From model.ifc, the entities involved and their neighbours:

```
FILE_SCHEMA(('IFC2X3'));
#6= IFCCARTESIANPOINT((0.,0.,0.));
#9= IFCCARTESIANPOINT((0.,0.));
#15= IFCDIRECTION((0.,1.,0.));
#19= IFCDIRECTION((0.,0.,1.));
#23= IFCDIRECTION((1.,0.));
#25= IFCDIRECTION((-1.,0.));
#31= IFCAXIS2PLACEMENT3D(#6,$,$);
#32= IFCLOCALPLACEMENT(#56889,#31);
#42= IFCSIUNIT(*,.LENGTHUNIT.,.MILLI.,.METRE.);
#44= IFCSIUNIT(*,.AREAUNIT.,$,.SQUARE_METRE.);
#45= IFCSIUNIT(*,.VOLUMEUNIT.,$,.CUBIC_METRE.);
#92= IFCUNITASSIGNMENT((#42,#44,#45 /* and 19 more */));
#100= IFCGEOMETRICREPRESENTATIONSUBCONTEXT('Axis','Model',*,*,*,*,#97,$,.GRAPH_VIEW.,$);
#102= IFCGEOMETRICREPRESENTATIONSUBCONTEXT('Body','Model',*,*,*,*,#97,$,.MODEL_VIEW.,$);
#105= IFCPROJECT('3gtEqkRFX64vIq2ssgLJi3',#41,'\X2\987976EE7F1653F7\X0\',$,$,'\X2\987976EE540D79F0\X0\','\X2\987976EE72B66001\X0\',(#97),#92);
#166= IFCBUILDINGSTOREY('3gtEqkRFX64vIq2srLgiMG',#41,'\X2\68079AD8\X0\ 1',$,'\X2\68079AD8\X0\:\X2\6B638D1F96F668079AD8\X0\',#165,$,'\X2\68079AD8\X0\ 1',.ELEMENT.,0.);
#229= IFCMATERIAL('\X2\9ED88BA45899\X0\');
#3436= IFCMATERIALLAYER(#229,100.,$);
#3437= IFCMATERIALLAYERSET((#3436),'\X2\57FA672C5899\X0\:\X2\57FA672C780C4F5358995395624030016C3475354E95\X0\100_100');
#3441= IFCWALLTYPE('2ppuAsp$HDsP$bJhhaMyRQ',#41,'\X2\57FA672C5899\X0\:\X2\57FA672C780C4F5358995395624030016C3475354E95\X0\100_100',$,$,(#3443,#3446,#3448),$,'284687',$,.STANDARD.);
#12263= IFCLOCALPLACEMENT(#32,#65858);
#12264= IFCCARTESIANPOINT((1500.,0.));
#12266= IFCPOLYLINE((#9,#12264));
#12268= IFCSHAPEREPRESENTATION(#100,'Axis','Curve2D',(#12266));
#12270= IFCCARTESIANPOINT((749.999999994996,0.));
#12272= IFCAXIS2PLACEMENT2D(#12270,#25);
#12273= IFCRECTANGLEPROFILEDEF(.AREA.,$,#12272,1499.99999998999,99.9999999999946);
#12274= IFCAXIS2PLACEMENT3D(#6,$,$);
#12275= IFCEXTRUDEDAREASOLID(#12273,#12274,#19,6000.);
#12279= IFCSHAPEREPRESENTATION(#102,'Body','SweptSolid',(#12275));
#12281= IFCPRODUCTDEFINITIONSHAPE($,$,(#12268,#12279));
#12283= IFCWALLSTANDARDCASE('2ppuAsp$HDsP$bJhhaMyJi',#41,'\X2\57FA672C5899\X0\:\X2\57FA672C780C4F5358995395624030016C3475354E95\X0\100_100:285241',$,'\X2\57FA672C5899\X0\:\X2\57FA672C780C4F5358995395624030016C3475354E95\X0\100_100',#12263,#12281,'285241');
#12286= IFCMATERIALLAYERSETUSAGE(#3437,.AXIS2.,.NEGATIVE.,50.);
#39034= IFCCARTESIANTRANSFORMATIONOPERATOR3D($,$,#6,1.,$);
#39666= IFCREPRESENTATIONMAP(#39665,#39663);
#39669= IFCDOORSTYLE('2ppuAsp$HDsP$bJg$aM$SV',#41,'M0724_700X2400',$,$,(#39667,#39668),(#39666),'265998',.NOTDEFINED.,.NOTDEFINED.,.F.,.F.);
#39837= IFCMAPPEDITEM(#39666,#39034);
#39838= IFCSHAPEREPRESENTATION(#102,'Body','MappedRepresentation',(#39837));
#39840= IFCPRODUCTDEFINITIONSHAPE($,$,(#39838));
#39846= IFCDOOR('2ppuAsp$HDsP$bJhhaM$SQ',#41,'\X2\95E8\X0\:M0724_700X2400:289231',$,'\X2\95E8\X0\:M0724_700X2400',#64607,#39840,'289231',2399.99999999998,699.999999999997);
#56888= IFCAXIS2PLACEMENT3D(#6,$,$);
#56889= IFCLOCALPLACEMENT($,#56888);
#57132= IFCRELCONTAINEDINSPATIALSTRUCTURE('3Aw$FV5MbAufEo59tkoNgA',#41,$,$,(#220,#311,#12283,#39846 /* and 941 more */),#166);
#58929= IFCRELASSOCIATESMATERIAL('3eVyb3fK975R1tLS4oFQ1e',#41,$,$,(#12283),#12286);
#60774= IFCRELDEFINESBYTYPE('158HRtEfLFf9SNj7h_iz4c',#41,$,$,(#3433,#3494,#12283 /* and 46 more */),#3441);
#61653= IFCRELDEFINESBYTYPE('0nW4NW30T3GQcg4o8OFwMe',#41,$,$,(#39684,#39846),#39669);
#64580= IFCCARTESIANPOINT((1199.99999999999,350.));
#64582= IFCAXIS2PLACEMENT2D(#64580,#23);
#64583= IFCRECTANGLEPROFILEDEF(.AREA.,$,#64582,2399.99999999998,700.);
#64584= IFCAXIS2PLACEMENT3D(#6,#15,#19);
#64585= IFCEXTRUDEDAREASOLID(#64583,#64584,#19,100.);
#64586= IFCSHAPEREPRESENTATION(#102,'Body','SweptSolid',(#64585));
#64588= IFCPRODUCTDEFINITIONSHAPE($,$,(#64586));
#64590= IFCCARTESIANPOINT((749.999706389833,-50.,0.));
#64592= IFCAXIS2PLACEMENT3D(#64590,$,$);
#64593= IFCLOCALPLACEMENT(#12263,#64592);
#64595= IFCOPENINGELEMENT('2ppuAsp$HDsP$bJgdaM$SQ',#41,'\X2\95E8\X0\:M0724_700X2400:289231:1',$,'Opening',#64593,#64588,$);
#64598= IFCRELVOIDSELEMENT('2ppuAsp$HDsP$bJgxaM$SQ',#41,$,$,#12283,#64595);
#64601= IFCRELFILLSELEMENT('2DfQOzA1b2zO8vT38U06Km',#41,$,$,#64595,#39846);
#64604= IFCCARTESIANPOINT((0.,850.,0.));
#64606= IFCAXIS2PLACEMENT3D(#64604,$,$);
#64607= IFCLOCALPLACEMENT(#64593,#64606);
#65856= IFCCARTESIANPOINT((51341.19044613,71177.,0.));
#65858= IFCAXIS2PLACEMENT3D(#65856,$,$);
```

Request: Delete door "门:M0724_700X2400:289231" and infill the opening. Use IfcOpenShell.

```python
import ifcopenshell
import ifcopenshell.api.feature
import ifcopenshell.api.root
import ifcopenshell.geom
import ifcopenshell.util.shape

model = ifcopenshell.open("model.ifc")
settings = ifcopenshell.geom.settings()


def volume(element):
    """Net volume in cubic metres, openings subtracted."""
    shape = ifcopenshell.geom.create_shape(settings, element)
    return ifcopenshell.util.shape.get_volume(shape.geometry)


door = model.by_guid("2ppuAsp$HDsP$bJhhaM$SQ")
opening = door.FillsVoids[0].RelatingOpeningElement
wall = opening.VoidsElements[0].RelatingBuildingElement
before = volume(wall)

ifcopenshell.api.root.remove_product(model, product=door)
ifcopenshell.api.feature.remove_feature(model, feature=opening)

after = volume(wall)

print(f"wall volume {before:.3f} -> {after:.3f} m3")

model.write("model_rev.ifc")
```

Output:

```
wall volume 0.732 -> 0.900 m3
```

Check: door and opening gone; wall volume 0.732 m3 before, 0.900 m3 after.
